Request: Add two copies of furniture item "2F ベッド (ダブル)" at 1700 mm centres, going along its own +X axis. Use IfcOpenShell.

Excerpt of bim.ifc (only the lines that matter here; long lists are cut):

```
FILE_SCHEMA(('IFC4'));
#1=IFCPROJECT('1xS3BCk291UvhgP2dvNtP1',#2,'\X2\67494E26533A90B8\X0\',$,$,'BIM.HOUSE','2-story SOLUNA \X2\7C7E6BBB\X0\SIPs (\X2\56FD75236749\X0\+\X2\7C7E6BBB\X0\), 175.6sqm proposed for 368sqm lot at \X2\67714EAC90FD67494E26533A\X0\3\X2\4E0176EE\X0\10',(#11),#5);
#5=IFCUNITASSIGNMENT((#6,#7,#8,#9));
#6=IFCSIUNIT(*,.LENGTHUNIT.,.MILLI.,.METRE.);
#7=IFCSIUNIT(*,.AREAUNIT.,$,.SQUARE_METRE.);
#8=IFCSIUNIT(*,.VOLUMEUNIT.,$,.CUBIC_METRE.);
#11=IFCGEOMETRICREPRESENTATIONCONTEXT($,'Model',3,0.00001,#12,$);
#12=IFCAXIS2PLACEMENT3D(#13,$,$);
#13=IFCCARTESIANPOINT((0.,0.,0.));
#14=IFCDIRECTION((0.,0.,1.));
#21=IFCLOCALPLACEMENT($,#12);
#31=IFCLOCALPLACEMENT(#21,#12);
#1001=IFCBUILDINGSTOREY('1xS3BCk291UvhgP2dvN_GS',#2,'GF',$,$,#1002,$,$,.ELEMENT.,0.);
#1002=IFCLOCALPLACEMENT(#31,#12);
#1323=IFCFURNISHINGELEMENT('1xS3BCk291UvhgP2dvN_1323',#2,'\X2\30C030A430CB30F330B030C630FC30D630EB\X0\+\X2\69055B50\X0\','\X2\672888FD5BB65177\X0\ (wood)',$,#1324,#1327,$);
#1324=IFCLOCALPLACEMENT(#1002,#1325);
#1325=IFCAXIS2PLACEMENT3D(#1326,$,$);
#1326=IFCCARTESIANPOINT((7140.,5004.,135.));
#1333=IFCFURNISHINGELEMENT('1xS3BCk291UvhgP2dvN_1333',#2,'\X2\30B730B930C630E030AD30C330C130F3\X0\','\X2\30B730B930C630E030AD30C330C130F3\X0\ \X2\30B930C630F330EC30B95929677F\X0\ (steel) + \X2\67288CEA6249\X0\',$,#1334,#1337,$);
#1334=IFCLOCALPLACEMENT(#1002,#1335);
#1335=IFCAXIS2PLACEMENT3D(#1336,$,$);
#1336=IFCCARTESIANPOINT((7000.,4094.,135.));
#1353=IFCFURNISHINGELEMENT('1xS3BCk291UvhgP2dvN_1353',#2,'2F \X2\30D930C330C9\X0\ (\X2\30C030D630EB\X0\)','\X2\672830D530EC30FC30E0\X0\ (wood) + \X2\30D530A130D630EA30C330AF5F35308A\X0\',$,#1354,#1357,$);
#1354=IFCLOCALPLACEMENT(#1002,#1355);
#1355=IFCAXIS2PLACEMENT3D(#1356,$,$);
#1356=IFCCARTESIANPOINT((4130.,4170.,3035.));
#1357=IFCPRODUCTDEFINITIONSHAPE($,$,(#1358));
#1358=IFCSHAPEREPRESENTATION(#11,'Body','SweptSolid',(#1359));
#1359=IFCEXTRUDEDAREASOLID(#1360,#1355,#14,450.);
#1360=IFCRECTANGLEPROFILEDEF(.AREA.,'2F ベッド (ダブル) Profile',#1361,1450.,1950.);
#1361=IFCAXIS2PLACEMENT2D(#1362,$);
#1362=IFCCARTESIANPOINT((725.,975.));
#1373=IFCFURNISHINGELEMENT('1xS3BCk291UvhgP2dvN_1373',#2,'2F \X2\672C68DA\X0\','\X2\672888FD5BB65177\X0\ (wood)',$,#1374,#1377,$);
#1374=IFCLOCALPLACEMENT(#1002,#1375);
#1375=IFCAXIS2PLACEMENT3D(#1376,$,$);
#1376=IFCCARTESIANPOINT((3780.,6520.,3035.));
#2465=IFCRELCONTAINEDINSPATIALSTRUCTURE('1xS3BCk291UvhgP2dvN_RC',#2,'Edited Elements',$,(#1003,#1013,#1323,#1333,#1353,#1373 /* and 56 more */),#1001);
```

```python
import ifcopenshell
import ifcopenshell.api.geometry
import ifcopenshell.api.root
import ifcopenshell.util.element
import ifcopenshell.util.placement

model = ifcopenshell.open("bim.ifc")


def reuse_history(source, copy):
    """copy_class also copies each property set's owner history, people and application; keep the originals."""
    for rel in copy.IsDefinedBy:
        if rel.is_a("IfcRelDefinesByProperties") and (history := rel.RelatingPropertyDefinition.OwnerHistory):
            rel.RelatingPropertyDefinition.OwnerHistory = source.OwnerHistory
            ifcopenshell.util.element.remove_deep2(model, history)


source = model.by_guid("1xS3BCk291UvhgP2dvN_1353")
base = ifcopenshell.util.placement.get_local_placement(source.ObjectPlacement)
step = base[:3, 0] * 1700.0

for i in range(1, 3):
    copy = ifcopenshell.api.root.copy_class(model, product=source)
    copy.Representation = ifcopenshell.util.element.copy_deep(
        model, source.Representation, exclude=["IfcGeometricRepresentationContext", "IfcRepresentationMap"]
    )
    reuse_history(source, copy)
    matrix = base.copy()
    matrix[:3, 3] += i * step
    print("added at", matrix[:3, 3].round(3) + 0.0)
    ifcopenshell.api.geometry.edit_object_placement(model, product=copy, matrix=matrix, is_si=False)

model.write("bim_rev.ifc")
```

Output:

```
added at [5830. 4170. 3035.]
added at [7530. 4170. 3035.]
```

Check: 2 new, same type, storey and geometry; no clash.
